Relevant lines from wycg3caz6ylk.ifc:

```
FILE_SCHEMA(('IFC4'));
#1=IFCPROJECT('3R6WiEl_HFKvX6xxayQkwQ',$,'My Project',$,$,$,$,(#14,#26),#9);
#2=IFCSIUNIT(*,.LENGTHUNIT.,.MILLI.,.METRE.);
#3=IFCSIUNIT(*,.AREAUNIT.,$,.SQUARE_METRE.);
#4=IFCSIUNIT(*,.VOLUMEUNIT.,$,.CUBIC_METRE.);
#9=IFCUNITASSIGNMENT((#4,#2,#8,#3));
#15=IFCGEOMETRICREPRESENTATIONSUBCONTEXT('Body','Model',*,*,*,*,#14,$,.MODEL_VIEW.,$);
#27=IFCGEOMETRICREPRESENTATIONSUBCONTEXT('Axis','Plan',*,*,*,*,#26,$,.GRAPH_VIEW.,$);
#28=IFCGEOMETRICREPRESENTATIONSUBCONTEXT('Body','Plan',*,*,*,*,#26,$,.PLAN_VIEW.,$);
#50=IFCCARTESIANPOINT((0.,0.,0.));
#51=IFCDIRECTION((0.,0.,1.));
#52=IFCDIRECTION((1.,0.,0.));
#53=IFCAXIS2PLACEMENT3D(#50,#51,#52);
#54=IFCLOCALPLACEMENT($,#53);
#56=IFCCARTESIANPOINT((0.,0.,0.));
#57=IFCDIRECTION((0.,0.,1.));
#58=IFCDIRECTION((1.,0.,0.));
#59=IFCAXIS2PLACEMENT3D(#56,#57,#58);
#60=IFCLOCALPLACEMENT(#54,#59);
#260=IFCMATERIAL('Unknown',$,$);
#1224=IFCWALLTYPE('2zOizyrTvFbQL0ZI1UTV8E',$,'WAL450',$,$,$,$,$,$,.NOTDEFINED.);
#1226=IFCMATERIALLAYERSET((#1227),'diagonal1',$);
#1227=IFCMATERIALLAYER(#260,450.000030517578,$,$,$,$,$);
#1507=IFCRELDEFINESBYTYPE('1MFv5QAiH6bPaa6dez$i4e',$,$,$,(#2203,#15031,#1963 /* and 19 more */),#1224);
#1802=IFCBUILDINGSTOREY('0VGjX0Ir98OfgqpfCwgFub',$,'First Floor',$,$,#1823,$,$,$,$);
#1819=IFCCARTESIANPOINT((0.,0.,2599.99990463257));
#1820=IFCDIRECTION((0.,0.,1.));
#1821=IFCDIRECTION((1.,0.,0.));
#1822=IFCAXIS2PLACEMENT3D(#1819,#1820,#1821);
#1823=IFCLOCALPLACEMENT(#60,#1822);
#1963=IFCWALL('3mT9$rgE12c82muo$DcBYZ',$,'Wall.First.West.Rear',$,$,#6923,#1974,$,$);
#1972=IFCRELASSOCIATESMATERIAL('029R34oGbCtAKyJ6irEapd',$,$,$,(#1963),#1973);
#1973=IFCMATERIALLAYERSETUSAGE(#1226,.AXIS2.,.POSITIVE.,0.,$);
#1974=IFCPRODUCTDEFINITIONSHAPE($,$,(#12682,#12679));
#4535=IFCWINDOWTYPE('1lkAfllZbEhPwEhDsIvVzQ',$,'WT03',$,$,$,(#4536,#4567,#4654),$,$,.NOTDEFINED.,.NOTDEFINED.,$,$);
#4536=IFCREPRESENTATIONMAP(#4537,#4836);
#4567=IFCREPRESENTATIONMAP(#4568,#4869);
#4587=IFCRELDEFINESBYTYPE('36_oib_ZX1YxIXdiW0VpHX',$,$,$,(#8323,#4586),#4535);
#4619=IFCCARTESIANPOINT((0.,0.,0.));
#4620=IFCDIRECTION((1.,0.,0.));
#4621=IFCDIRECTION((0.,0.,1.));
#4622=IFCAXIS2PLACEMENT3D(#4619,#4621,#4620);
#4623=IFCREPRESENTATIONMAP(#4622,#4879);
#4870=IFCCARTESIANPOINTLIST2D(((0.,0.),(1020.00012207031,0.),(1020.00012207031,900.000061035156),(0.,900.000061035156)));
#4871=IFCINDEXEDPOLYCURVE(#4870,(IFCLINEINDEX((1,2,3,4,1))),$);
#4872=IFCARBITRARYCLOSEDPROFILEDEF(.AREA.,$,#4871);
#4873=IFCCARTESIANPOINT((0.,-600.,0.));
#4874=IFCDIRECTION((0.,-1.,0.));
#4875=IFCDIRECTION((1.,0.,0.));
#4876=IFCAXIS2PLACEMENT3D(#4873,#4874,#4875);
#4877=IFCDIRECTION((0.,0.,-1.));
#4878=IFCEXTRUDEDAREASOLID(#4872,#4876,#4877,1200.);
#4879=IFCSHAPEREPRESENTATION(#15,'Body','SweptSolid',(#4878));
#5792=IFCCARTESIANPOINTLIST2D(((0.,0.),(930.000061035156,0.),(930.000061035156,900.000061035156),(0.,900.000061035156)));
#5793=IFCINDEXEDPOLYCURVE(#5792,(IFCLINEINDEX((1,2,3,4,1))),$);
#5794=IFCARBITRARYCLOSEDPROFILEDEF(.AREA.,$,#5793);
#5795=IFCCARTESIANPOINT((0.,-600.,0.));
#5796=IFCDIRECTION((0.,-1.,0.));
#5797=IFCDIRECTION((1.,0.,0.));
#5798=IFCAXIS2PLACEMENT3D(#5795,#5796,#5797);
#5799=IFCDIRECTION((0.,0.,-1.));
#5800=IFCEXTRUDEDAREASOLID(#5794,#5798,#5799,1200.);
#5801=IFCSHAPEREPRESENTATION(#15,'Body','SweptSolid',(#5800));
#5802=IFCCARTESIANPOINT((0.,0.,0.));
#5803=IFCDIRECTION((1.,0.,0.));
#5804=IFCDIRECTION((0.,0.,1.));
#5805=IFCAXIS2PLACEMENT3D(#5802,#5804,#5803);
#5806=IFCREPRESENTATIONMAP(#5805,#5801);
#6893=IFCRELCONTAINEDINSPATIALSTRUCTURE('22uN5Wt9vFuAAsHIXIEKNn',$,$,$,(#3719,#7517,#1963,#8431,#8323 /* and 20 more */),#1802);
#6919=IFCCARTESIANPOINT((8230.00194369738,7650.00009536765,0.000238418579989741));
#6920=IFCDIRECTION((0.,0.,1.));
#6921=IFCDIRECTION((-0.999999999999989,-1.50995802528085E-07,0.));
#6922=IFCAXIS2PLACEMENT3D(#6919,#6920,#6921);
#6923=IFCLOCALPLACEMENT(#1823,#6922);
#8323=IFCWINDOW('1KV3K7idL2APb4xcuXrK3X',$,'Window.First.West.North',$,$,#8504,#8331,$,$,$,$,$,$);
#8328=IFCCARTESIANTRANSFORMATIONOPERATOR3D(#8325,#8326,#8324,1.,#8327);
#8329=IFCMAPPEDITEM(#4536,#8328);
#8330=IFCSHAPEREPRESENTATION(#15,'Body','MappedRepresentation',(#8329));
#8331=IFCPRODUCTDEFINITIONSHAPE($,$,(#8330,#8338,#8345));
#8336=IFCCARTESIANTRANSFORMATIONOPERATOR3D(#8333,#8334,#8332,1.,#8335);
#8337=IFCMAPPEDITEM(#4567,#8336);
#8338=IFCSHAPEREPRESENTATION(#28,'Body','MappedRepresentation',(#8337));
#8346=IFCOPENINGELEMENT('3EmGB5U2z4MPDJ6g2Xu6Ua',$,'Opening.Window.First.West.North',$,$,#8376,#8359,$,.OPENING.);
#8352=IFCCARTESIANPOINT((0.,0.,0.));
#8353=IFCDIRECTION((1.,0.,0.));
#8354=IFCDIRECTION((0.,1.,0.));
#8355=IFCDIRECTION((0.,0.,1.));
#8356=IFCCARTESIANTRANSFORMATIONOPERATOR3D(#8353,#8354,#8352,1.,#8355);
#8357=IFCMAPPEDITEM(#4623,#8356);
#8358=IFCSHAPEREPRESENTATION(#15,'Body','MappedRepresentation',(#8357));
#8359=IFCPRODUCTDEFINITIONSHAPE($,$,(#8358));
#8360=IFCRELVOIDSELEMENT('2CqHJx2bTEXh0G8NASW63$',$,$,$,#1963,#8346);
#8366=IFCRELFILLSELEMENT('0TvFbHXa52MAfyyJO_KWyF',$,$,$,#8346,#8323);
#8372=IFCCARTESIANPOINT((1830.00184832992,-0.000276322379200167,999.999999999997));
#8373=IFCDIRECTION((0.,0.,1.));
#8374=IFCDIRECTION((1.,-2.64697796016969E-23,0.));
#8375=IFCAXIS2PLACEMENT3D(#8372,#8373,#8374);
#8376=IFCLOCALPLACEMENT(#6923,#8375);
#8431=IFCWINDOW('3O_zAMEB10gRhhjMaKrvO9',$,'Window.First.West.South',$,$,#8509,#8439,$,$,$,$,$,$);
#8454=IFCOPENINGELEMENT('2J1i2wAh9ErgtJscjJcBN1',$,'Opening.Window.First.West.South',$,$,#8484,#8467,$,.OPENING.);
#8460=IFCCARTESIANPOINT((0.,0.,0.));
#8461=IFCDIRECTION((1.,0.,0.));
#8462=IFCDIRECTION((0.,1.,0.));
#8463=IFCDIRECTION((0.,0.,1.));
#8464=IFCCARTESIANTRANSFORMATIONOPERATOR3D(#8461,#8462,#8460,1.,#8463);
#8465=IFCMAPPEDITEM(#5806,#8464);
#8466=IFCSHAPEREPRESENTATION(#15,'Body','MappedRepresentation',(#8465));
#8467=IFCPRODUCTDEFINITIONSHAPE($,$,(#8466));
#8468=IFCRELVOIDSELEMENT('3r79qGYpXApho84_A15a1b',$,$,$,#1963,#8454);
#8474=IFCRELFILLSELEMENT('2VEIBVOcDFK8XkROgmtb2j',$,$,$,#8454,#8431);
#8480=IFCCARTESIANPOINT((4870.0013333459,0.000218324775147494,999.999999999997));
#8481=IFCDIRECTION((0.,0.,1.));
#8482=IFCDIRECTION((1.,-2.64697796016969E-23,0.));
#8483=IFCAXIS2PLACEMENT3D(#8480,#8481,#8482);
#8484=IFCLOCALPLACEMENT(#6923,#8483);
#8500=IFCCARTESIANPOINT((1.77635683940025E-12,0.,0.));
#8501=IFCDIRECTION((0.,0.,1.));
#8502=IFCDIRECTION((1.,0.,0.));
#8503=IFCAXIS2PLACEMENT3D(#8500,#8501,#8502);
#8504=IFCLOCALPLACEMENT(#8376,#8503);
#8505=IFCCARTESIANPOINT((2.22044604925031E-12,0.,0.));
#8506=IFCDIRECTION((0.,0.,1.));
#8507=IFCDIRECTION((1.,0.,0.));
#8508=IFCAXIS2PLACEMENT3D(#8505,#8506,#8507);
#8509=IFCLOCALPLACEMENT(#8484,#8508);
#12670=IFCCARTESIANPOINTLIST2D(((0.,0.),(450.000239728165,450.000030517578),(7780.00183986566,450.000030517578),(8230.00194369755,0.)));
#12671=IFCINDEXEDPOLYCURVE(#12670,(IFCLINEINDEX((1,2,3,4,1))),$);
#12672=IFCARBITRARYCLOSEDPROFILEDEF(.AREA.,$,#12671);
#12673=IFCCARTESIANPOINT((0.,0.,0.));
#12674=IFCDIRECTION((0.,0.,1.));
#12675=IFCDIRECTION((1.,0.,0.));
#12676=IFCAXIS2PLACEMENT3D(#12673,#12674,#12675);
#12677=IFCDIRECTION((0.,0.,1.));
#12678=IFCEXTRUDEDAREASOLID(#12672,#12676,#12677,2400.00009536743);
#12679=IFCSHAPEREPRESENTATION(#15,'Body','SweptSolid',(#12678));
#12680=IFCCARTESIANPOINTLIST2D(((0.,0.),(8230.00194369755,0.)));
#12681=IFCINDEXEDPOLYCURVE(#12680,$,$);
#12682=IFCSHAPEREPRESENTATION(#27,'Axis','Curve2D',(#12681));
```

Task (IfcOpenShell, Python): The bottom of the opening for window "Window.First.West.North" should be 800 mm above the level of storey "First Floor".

```python
import numpy as np
import ifcopenshell
import ifcopenshell.api.geometry
import ifcopenshell.geom
import ifcopenshell.util.element
import ifcopenshell.util.placement
import ifcopenshell.util.shape
import ifcopenshell.util.unit

model = ifcopenshell.open("wycg3caz6ylk.ifc")
unit_scale = ifcopenshell.util.unit.calculate_unit_scale(model)

window = model.by_guid("1KV3K7idL2APb4xcuXrK3X")
opening = window.FillsVoids[0].RelatingOpeningElement
storey = ifcopenshell.util.element.get_container(window, ifc_class="IfcBuildingStorey")
level = ifcopenshell.util.placement.get_local_placement(storey.ObjectPlacement)[2, 3]

# The opening's origin need not be at the sill, so measure its lowest point.
shape = ifcopenshell.geom.create_shape(ifcopenshell.geom.settings(), opening)
bottom = ifcopenshell.util.shape.get_shape_bottom_elevation(shape, shape.geometry) / unit_scale
dz = level + 0.8 / unit_scale - bottom

shift = np.array([0.0, 0.0, dz])
# The window is placed relative to its opening, so it follows when the opening moves.
matrix = ifcopenshell.util.placement.get_local_placement(opening.ObjectPlacement)
matrix[:3, 3] += shift
ifcopenshell.api.geometry.edit_object_placement(
    model, product=opening, matrix=matrix, is_si=False, should_transform_children=True
)

print(f"moved by {dz * unit_scale:+.3f} m")

model.write("wycg3caz6ylk_updated.ifc")
```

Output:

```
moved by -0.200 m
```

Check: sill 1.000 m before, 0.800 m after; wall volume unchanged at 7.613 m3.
